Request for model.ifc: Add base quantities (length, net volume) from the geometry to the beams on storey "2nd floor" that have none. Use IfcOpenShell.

First a look at what the model holds.

```python
import ifcopenshell
import ifcopenshell.util.element
import ifcopenshell.util.unit

model = ifcopenshell.open("model.ifc")
print(model.schema)
for unit_type in ("LENGTHUNIT", "AREAUNIT", "VOLUMEUNIT"):
    print(unit_type, ifcopenshell.util.unit.calculate_unit_scale(model, unit_type))
storey = next(s for s in model.by_type("IfcBuildingStorey") if s.Name == "2nd floor")
beams = [e for e in ifcopenshell.util.element.get_decomposition(storey) if e.is_a("IfcBeam")]
for e in sorted(beams, key=lambda e: e.id()):
    print(e.id(), e.is_a(), e.Name, list(ifcopenshell.util.element.get_psets(e, qtos_only=True)), sep=" | ")
```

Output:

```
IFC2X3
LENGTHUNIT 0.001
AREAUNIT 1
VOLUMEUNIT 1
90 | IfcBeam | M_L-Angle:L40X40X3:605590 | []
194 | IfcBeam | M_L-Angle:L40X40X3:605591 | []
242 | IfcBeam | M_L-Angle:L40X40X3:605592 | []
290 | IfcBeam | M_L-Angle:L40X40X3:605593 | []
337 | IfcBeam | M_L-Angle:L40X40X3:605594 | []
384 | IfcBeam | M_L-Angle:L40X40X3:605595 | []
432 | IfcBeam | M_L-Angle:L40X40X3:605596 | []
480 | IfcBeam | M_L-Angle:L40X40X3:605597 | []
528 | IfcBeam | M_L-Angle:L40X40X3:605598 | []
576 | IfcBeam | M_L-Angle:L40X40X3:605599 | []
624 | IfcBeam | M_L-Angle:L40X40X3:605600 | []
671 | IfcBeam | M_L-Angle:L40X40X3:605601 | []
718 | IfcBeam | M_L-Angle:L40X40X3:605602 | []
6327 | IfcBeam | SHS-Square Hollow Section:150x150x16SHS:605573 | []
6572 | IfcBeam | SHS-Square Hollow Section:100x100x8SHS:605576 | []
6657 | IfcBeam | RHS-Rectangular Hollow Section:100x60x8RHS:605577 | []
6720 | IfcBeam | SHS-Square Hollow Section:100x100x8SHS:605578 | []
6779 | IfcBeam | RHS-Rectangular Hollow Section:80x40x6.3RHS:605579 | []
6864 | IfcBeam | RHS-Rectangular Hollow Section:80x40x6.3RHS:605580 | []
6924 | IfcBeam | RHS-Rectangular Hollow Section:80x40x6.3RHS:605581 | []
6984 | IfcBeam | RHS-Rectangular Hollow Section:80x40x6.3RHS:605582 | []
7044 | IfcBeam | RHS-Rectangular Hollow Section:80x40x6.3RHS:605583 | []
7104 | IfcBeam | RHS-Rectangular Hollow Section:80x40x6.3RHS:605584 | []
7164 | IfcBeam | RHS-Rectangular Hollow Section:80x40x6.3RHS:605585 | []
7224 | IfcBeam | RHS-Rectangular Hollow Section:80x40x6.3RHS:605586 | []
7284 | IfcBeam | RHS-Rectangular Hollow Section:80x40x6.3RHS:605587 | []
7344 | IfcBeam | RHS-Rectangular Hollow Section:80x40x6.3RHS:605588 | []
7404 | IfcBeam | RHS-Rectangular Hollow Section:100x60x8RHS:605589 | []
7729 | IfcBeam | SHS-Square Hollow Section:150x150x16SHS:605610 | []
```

```python
import ifcopenshell
import ifcopenshell.api.pset
import ifcopenshell.geom
import ifcopenshell.util.element
import ifcopenshell.util.shape
import ifcopenshell.util.unit

model = ifcopenshell.open("model.ifc")
unit_scale = ifcopenshell.util.unit.calculate_unit_scale(model)
volume_scale = ifcopenshell.util.unit.calculate_unit_scale(model, "VOLUMEUNIT")
settings = ifcopenshell.geom.settings()

storey = next(s for s in model.by_type("IfcBuildingStorey") if s.Name == "2nd floor")
beams = [e for e in ifcopenshell.util.element.get_decomposition(storey) if e.is_a("IfcBeam")]

for e in sorted(beams, key=lambda e: e.id()):
    if ifcopenshell.util.element.get_psets(e, qtos_only=True, should_inherit=False):
        continue
    # Geometry comes back in metres, in the element's own axes.
    shape = ifcopenshell.geom.create_shape(settings, e)
    values = {
        "Length": ifcopenshell.util.shape.get_max_xyz(shape.geometry) / unit_scale,
        "NetVolume": ifcopenshell.util.shape.get_volume(shape.geometry) / volume_scale,
    }
    qto = ifcopenshell.api.pset.add_qto(model, product=e, name="BaseQuantities")
    ifcopenshell.api.pset.edit_qto(model, qto=qto, properties=values)
    print(e.id(), {k: round(v, 3) for k, v in values.items()})

model.write("model_edited.ifc")
```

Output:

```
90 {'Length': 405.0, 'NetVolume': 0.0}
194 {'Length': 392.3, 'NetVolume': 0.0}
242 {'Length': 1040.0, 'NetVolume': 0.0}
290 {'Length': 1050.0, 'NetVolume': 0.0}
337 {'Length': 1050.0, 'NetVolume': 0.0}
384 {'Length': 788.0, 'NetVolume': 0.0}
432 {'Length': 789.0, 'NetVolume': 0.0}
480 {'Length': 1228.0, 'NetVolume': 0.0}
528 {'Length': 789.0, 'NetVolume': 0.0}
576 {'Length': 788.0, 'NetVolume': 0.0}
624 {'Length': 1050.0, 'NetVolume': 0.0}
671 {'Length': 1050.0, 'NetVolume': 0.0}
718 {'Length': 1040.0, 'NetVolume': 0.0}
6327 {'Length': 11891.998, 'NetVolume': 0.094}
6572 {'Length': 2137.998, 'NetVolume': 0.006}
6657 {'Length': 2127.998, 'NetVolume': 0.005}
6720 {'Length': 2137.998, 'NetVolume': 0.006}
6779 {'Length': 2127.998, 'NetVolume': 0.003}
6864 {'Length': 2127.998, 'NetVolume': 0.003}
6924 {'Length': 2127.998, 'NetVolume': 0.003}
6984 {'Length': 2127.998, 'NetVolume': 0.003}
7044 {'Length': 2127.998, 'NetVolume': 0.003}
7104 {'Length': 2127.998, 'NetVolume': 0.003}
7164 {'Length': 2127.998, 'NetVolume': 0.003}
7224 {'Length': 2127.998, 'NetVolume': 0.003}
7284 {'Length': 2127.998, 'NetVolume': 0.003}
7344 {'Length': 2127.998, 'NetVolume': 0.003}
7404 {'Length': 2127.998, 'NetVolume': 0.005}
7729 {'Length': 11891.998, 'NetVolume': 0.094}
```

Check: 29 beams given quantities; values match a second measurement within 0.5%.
